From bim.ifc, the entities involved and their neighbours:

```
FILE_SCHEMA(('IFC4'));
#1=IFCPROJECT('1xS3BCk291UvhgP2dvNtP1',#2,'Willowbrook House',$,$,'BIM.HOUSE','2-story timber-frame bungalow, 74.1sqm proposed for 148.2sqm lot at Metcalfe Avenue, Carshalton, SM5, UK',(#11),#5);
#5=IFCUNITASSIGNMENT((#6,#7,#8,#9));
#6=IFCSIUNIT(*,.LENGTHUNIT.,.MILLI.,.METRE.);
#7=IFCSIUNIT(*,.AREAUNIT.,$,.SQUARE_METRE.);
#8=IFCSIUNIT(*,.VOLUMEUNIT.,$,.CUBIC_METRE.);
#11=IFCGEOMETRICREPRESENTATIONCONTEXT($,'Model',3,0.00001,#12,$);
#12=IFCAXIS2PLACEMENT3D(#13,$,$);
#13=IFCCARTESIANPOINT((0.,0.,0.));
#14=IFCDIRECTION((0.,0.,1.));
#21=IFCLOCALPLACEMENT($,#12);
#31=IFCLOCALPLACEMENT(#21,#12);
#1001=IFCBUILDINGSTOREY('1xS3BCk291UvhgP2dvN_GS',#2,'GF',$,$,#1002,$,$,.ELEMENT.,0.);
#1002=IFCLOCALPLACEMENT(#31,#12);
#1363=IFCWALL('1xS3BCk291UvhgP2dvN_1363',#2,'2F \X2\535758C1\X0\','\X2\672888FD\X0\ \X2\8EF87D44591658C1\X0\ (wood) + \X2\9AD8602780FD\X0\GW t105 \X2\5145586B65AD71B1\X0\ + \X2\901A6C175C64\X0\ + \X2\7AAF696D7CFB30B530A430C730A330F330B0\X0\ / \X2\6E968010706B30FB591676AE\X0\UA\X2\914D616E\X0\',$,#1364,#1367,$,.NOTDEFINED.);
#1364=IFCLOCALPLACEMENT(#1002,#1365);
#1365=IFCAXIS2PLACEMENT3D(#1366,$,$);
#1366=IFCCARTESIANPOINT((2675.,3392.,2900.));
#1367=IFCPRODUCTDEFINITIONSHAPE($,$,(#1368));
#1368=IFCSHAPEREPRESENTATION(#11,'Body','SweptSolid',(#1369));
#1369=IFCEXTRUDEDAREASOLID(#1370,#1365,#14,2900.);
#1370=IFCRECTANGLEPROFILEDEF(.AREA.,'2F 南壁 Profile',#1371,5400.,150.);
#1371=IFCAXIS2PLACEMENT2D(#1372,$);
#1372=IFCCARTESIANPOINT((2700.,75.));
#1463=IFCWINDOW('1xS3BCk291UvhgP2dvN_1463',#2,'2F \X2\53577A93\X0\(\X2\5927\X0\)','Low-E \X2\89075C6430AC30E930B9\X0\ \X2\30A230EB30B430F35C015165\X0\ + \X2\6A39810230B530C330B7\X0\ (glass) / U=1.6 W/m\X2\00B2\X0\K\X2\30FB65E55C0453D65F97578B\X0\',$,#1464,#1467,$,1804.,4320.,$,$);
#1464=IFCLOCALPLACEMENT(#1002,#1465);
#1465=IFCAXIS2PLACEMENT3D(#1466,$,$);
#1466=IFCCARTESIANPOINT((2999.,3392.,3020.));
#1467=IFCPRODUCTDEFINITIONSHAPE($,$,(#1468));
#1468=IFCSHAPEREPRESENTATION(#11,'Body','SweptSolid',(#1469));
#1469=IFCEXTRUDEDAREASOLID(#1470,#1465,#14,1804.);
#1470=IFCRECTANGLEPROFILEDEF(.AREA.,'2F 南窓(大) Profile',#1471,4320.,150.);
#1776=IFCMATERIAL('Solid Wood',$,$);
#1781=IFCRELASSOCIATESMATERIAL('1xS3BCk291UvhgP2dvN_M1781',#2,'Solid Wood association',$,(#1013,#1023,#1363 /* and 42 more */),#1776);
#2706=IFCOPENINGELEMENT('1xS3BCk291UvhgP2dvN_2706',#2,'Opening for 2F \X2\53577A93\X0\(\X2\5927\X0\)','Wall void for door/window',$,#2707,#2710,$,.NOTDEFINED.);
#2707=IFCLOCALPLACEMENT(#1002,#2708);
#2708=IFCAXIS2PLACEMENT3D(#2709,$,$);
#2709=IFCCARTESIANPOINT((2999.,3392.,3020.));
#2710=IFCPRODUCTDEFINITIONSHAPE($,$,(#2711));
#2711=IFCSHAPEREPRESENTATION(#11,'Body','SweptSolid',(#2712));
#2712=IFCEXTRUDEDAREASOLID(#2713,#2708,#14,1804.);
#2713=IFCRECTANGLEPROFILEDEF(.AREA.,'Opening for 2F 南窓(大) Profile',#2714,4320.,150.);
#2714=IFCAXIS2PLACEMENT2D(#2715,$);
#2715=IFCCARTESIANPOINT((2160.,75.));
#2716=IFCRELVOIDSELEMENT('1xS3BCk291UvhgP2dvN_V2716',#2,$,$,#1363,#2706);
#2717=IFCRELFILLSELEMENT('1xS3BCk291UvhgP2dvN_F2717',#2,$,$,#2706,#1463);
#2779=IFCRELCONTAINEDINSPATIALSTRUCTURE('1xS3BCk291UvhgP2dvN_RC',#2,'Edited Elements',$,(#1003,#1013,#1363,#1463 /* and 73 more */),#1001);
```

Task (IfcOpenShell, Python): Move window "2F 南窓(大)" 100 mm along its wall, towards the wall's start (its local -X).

```python
import ifcopenshell
import ifcopenshell.api.geometry
import ifcopenshell.util.placement

model = ifcopenshell.open("bim.ifc")

window = model.by_id(1463)
opening = window.FillsVoids[0].RelatingOpeningElement
wall = opening.VoidsElements[0].RelatingBuildingElement

wall_matrix = ifcopenshell.util.placement.get_local_placement(wall.ObjectPlacement)
shift = wall_matrix[:3, 0] * -100.0
before = ifcopenshell.util.placement.get_local_placement(window.ObjectPlacement)[:3, 3].copy()

# The window is not placed relative to its opening, so move both.
for product in (opening, window):
    matrix = ifcopenshell.util.placement.get_local_placement(product.ObjectPlacement)
    matrix[:3, 3] += shift
    ifcopenshell.api.geometry.edit_object_placement(model, product=product, matrix=matrix, is_si=False)

after = ifcopenshell.util.placement.get_local_placement(window.ObjectPlacement)[:3, 3]
print("window moved by", (after - before).round(3) + 0.0)

model.write("bim_edited.ifc")
```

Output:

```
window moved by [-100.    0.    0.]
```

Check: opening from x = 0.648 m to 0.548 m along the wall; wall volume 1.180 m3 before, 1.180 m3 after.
